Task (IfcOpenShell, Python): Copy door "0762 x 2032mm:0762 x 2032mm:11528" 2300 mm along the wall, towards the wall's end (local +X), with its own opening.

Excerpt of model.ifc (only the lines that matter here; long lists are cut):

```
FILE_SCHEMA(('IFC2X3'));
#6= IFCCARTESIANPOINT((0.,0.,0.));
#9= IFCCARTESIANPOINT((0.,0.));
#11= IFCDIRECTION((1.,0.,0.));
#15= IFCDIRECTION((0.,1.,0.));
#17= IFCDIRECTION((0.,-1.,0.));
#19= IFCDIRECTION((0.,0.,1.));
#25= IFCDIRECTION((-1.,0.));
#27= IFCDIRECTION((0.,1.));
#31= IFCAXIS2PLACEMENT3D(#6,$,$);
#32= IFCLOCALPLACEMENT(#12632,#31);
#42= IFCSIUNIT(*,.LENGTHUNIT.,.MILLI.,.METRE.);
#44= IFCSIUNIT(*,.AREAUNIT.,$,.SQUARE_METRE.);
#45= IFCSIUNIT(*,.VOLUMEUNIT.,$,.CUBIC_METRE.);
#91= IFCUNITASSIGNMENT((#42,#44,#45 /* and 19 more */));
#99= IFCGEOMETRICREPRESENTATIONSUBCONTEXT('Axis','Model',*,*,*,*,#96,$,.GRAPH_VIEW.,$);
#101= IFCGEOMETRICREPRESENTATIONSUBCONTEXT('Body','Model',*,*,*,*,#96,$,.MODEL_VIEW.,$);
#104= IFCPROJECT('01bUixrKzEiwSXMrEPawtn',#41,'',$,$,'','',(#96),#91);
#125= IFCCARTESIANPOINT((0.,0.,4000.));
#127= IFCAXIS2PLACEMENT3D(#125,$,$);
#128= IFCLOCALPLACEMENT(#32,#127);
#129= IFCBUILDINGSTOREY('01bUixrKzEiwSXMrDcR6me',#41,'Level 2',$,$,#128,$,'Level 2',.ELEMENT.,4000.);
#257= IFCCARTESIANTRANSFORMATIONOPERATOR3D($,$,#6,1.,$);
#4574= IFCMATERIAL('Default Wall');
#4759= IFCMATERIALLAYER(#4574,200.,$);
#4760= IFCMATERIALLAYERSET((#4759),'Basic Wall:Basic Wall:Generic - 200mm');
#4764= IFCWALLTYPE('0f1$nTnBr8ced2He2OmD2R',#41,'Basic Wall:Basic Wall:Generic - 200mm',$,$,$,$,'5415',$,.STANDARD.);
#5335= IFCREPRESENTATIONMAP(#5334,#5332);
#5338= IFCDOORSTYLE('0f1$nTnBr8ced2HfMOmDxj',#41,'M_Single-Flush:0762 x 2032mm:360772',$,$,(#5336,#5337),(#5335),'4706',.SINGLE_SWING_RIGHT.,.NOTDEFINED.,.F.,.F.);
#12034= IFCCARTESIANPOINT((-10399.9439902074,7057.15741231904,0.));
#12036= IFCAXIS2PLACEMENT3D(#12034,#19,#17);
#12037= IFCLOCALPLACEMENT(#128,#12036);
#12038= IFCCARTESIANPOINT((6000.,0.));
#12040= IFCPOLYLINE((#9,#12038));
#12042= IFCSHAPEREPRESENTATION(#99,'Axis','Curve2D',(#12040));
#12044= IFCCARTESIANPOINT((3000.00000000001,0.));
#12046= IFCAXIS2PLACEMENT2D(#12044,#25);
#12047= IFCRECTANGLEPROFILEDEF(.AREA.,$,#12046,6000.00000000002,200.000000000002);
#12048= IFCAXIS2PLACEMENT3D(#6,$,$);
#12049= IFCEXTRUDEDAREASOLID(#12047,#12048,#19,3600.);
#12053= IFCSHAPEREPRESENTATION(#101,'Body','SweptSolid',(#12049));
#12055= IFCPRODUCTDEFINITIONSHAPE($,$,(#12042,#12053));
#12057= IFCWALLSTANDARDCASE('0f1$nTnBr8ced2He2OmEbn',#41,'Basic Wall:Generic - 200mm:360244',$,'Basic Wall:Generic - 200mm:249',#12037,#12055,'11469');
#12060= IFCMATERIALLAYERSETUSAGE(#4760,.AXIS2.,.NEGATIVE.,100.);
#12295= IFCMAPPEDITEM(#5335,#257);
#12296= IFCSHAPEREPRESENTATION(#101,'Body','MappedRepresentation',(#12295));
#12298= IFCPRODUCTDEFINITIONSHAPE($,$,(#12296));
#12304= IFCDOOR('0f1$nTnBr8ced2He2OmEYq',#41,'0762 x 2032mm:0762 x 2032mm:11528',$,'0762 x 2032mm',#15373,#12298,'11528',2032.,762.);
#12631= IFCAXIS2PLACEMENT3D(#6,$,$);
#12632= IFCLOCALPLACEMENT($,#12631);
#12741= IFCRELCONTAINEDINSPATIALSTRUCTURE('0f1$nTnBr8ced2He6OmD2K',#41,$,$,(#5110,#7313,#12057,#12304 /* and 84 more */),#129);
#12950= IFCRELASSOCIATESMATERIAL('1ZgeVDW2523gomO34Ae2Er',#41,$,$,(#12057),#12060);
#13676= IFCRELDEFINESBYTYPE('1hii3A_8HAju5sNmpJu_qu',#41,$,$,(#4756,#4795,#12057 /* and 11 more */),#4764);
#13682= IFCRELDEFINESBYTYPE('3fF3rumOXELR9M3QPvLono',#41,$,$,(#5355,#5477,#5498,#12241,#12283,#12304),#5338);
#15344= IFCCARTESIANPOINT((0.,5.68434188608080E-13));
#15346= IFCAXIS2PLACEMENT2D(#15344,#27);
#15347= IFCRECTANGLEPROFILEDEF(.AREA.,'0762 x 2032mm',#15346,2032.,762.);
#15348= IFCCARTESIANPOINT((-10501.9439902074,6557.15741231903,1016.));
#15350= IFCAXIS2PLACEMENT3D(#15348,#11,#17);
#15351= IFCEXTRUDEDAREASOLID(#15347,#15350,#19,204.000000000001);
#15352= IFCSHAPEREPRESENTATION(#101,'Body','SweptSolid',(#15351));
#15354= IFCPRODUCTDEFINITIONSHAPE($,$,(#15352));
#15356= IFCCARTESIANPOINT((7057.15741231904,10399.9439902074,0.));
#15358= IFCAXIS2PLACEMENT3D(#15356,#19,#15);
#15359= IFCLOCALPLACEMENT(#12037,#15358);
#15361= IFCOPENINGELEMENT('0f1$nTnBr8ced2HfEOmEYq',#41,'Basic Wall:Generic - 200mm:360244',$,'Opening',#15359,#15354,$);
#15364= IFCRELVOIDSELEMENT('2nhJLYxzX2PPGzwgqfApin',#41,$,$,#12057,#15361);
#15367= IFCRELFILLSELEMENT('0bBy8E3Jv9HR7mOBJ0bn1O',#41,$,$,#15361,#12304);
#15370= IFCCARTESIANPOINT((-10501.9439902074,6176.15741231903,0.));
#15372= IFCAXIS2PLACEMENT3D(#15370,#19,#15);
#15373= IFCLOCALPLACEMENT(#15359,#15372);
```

```python
import ifcopenshell
import ifcopenshell.api.feature
import ifcopenshell.api.geometry
import ifcopenshell.api.root
import ifcopenshell.geom
import ifcopenshell.util.element
import ifcopenshell.util.placement
import ifcopenshell.util.shape
import ifcopenshell.util.unit

model = ifcopenshell.open("model.ifc")
unit_scale = ifcopenshell.util.unit.calculate_unit_scale(model)
settings = ifcopenshell.geom.settings()


def volume(element):
    """Net volume in cubic metres, openings subtracted."""
    shape = ifcopenshell.geom.create_shape(settings, element)
    return ifcopenshell.util.shape.get_volume(shape.geometry)


def reuse_history(source, copy):
    """copy_class also copies each property set's owner history, people and application; keep the originals."""
    for rel in copy.IsDefinedBy:
        if rel.is_a("IfcRelDefinesByProperties") and (history := rel.RelatingPropertyDefinition.OwnerHistory):
            rel.RelatingPropertyDefinition.OwnerHistory = source.OwnerHistory
            ifcopenshell.util.element.remove_deep2(model, history)


door = model.by_guid("0f1$nTnBr8ced2He2OmEYq")
opening = door.FillsVoids[0].RelatingOpeningElement
wall = opening.VoidsElements[0].RelatingBuildingElement
before = volume(wall)
shift = ifcopenshell.util.placement.get_local_placement(wall.ObjectPlacement)[:3, 0] * 2.3 / unit_scale

# copy_class copies the void relationship, type, container and properties, but no geometry.
new_opening = ifcopenshell.api.root.copy_class(model, product=opening)
new_opening.Representation = ifcopenshell.util.element.copy_deep(
    model, opening.Representation, exclude=["IfcGeometricRepresentationContext", "IfcRepresentationMap"]
)
new_opening.Name = "Basic Wall:Generic - 200mm"
new_door = ifcopenshell.api.root.copy_class(model, product=door)
new_door.Representation = ifcopenshell.util.element.copy_deep(
    model, door.Representation, exclude=["IfcGeometricRepresentationContext", "IfcRepresentationMap"]
)
new_door.Name = "0762 x 2032mm:0762 x 2032mm"
new_door.Tag = None
reuse_history(door, new_door)
fills = ifcopenshell.api.feature.add_filling(model, opening=new_opening, element=new_door)
fills.OwnerHistory = new_door.OwnerHistory  # required in IFC2X3

for old, new in ((opening, new_opening), (door, new_door)):
    matrix = ifcopenshell.util.placement.get_local_placement(old.ObjectPlacement)
    matrix[:3, 3] += shift
    ifcopenshell.api.geometry.edit_object_placement(model, product=new, matrix=matrix, is_si=False)

after = volume(wall)

print(f"wall volume {before:.3f} -> {after:.3f} m3")

model.write("model_v2.ifc")
```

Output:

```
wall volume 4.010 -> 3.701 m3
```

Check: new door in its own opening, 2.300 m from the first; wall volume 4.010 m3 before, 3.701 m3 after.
